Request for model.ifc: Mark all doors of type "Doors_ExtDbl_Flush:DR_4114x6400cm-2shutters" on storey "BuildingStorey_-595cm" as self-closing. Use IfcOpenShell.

First a look at what the model holds.

```python
import ifcopenshell
import ifcopenshell.util.element

model = ifcopenshell.open("model.ifc")
print(model.schema)
storey = next(s for s in model.by_type("IfcBuildingStorey") if s.Name == "BuildingStorey_-595cm")
doors = [e for e in ifcopenshell.util.element.get_decomposition(storey) if e.is_a("IfcDoor")]
seen = {}
for e in doors:
    element_type = ifcopenshell.util.element.get_type(e)
    key = (element_type.Name if element_type != e and element_type else None, ifcopenshell.util.element.get_pset(e, "Pset_DoorCommon", "SelfClosing"))
    seen[key] = seen.get(key, 0) + 1
for (name, value), count in sorted(seen.items(), key=str):
    print(count, "x", name, "|", value)
```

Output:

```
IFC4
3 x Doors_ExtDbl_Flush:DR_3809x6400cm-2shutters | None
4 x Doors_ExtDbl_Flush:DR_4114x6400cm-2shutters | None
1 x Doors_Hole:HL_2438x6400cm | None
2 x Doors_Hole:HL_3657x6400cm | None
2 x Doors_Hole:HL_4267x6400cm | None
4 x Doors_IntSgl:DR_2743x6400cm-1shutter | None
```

```python
import ifcopenshell
import ifcopenshell.api.pset
import ifcopenshell.util.element

model = ifcopenshell.open("model.ifc")

storey = next(s for s in model.by_type("IfcBuildingStorey") if s.Name == "BuildingStorey_-595cm")
doors = [e for e in ifcopenshell.util.element.get_decomposition(storey) if e.is_a("IfcDoor")]

count = 0
for e in doors:
    element_type = ifcopenshell.util.element.get_type(e)
    if element_type in (None, e) or element_type.Name != "Doors_ExtDbl_Flush:DR_4114x6400cm-2shutters":
        continue
    # add_pset returns the element's existing set when there is one.
    pset = ifcopenshell.api.pset.add_pset(model, product=e, name="Pset_DoorCommon")
    ifcopenshell.api.pset.edit_pset(model, pset=pset, properties={"SelfClosing": True})
    count += 1

print(count, "doors updated")

model.write("model_edited.ifc")
```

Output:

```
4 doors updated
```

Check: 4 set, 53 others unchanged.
